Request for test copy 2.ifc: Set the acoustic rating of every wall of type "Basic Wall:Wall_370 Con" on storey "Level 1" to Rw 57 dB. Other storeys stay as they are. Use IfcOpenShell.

First a look at what the model holds.

```python
import ifcopenshell
import ifcopenshell.util.element

model = ifcopenshell.open("test copy 2.ifc")
print(model.schema)
storey = next(s for s in model.by_type("IfcBuildingStorey") if s.Name == "Level 1")
walls = [e for e in ifcopenshell.util.element.get_decomposition(storey) if e.is_a("IfcWall")]
seen = {}
for e in walls:
    element_type = ifcopenshell.util.element.get_type(e)
    key = (element_type.Name if element_type != e and element_type else None, ifcopenshell.util.element.get_pset(e, "Pset_WallCommon", "AcousticRating"))
    seen[key] = seen.get(key, 0) + 1
for (name, value), count in sorted(seen.items(), key=str):
    print(count, "x", name, "|", value)
```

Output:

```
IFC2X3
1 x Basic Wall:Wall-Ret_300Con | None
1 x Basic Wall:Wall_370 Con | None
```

```python
import ifcopenshell
import ifcopenshell.api.pset
import ifcopenshell.util.element

model = ifcopenshell.open("test copy 2.ifc")

storey = next(s for s in model.by_type("IfcBuildingStorey") if s.Name == "Level 1")
walls = [e for e in ifcopenshell.util.element.get_decomposition(storey) if e.is_a("IfcWall")]

count = 0
for e in walls:
    element_type = ifcopenshell.util.element.get_type(e)
    if element_type in (None, e) or element_type.Name != "Basic Wall:Wall_370 Con":
        continue
    # add_pset returns the element's existing set when there is one.
    pset = ifcopenshell.api.pset.add_pset(model, product=e, name="Pset_WallCommon")
    ifcopenshell.api.pset.edit_pset(model, pset=pset, properties={"AcousticRating": "Rw 57 dB"})
    count += 1

print(count, "walls updated")

model.write("test copy 2_updated.ifc")
```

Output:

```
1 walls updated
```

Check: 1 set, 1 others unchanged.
